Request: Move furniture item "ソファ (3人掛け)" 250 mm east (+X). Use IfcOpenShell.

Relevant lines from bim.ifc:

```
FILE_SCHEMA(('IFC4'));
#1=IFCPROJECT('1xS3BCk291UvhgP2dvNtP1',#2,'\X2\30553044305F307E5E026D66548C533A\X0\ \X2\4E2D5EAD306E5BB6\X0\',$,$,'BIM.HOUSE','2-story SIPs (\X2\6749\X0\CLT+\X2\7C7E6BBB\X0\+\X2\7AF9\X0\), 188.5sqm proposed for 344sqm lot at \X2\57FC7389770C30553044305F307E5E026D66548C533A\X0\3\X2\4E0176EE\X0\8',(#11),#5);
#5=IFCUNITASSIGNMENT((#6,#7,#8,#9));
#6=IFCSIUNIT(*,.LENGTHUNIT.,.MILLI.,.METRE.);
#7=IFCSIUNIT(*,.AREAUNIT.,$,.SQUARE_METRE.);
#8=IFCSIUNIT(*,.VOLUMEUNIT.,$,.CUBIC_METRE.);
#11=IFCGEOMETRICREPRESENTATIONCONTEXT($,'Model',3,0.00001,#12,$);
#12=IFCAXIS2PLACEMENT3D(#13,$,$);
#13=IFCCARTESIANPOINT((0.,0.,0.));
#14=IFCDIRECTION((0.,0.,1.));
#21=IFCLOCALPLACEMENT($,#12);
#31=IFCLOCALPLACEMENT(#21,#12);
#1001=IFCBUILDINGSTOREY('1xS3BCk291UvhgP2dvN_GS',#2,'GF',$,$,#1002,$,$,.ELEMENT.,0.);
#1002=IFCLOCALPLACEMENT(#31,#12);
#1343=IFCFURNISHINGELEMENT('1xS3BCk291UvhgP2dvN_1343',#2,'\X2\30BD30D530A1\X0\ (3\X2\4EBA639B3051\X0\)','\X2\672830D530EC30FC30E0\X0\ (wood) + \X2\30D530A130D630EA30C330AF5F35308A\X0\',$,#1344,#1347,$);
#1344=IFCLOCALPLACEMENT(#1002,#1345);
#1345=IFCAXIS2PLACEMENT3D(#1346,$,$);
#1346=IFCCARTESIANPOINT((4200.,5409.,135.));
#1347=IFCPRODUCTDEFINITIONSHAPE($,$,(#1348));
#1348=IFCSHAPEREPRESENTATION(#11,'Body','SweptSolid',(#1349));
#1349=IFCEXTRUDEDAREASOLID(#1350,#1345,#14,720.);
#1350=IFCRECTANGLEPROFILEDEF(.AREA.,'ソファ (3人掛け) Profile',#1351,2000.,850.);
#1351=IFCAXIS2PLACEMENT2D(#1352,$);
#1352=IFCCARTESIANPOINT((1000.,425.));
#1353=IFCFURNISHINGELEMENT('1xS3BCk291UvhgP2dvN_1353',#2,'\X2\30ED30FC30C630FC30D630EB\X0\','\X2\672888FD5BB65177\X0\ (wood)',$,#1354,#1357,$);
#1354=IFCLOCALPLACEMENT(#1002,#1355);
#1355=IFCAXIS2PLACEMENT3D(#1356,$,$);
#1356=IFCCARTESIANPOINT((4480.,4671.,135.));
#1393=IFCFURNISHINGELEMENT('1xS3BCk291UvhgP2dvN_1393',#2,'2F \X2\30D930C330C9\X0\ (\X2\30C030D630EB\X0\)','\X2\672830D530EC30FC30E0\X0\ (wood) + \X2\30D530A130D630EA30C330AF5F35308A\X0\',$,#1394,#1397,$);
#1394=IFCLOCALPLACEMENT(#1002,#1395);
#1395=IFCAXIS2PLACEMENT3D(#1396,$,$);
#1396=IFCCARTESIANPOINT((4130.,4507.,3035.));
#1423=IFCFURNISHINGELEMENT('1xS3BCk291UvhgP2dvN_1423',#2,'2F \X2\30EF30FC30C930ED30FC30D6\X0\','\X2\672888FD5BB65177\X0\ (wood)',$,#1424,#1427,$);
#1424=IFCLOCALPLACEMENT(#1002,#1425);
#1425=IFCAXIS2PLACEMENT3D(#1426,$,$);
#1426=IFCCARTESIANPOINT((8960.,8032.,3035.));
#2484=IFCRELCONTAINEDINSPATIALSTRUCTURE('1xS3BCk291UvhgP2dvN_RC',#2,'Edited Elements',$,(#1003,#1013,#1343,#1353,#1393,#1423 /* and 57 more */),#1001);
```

```python
import ifcopenshell
import ifcopenshell.api.geometry
import ifcopenshell.util.placement
import ifcopenshell.util.unit

model = ifcopenshell.open("bim.ifc")
unit_scale = ifcopenshell.util.unit.calculate_unit_scale(model)

item = model.by_id(1343)
matrix = ifcopenshell.util.placement.get_local_placement(item.ObjectPlacement)
matrix[0, 3] += 0.25 / unit_scale
ifcopenshell.api.geometry.edit_object_placement(model, product=item, matrix=matrix, is_si=False)

print(ifcopenshell.util.placement.get_local_placement(item.ObjectPlacement).round(3) + 0.0)

model.write("bim_v2.ifc")
```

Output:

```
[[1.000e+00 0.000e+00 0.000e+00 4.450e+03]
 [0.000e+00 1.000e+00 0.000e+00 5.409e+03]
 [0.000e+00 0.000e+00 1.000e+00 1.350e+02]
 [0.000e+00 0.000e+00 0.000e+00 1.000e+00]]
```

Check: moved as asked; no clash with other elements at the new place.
